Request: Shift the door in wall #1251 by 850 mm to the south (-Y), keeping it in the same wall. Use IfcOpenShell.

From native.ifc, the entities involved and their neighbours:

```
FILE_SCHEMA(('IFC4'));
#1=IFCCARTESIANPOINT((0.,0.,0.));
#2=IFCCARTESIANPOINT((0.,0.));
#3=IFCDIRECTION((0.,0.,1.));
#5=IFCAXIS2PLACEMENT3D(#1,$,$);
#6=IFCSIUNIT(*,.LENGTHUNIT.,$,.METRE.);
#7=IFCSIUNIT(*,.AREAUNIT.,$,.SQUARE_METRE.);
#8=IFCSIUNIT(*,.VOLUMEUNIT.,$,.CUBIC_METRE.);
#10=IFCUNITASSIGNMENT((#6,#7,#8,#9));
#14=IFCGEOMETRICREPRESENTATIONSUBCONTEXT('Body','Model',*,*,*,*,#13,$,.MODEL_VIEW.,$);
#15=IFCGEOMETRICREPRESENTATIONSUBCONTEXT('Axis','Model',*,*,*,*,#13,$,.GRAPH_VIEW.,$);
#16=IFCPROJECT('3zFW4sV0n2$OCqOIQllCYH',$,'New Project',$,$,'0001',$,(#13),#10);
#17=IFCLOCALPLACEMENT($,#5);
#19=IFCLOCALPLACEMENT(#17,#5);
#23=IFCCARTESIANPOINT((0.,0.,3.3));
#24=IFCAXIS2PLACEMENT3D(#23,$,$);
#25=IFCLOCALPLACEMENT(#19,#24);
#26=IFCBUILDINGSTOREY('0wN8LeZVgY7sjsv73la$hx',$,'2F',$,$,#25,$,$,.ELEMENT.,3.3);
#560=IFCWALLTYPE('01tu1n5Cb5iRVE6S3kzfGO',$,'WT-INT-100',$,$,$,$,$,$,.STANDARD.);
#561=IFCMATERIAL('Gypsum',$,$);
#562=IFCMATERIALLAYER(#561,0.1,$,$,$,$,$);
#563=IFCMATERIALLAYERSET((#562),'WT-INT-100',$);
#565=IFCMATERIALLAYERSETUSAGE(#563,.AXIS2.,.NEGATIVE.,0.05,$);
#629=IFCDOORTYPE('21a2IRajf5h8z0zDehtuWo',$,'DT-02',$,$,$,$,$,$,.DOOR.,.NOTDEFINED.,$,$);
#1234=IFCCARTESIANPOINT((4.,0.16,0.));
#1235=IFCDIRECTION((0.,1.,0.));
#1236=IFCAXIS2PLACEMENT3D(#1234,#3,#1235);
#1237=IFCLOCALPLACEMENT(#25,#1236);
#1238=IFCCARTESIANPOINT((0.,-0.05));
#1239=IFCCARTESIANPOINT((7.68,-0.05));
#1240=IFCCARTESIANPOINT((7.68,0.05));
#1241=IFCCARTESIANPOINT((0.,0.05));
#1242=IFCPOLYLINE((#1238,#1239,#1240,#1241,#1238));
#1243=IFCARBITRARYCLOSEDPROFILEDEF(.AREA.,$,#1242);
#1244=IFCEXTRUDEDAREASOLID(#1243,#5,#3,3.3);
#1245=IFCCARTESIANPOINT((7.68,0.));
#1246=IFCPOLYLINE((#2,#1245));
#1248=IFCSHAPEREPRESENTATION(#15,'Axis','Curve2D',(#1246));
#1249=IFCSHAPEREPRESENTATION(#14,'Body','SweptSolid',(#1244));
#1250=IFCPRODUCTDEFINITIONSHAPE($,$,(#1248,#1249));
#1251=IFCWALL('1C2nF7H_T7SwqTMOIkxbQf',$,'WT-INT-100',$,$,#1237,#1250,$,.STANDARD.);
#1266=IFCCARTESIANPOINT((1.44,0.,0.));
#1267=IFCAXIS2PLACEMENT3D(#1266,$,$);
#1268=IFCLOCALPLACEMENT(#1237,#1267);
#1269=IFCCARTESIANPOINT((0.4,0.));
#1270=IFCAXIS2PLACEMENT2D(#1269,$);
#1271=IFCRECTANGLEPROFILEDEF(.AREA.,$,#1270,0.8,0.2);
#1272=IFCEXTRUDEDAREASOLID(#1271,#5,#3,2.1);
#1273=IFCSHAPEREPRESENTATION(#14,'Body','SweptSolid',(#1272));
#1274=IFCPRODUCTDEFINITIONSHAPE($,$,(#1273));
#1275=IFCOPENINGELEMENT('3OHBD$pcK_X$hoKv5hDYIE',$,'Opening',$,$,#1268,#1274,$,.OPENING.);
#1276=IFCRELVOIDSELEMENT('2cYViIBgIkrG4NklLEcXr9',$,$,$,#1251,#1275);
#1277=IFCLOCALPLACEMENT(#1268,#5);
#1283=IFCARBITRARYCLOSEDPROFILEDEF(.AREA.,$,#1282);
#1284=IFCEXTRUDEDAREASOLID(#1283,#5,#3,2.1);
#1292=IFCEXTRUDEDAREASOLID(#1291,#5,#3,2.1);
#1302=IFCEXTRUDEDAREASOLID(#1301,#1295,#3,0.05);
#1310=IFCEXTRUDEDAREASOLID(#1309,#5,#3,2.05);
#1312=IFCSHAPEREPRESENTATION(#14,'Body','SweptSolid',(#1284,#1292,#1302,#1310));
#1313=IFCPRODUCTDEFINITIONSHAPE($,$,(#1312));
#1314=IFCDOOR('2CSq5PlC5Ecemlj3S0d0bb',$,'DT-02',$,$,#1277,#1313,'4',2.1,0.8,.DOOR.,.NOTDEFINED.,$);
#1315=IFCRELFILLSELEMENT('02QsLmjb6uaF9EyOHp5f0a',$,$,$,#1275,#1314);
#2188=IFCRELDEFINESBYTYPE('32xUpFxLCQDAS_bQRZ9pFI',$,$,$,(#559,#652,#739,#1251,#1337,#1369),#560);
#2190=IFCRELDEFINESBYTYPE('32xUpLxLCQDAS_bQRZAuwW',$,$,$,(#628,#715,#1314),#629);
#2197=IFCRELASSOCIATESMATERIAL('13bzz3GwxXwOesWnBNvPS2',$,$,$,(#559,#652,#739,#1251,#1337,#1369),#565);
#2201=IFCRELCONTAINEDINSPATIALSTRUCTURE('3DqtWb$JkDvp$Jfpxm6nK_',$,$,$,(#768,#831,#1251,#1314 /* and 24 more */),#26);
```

```python
import ifcopenshell
import ifcopenshell.api.geometry
import ifcopenshell.util.placement

model = ifcopenshell.open("native.ifc")

door = model.by_id(1314)
opening = door.FillsVoids[0].RelatingOpeningElement
wall = opening.VoidsElements[0].RelatingBuildingElement

wall_matrix = ifcopenshell.util.placement.get_local_placement(wall.ObjectPlacement)
shift = wall_matrix[:3, 0] * -0.85
before = ifcopenshell.util.placement.get_local_placement(door.ObjectPlacement)[:3, 3].copy()

# The door is placed relative to its opening, so it follows when the opening moves.
matrix = ifcopenshell.util.placement.get_local_placement(opening.ObjectPlacement)
matrix[:3, 3] += shift
ifcopenshell.api.geometry.edit_object_placement(
    model, product=opening, matrix=matrix, is_si=False, should_transform_children=True
)

after = ifcopenshell.util.placement.get_local_placement(door.ObjectPlacement)[:3, 3]
print("door moved by", (after - before).round(3) + 0.0)

model.write("native_rev.ifc")
```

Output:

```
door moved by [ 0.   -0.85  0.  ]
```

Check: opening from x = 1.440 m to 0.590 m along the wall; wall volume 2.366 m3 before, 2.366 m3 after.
